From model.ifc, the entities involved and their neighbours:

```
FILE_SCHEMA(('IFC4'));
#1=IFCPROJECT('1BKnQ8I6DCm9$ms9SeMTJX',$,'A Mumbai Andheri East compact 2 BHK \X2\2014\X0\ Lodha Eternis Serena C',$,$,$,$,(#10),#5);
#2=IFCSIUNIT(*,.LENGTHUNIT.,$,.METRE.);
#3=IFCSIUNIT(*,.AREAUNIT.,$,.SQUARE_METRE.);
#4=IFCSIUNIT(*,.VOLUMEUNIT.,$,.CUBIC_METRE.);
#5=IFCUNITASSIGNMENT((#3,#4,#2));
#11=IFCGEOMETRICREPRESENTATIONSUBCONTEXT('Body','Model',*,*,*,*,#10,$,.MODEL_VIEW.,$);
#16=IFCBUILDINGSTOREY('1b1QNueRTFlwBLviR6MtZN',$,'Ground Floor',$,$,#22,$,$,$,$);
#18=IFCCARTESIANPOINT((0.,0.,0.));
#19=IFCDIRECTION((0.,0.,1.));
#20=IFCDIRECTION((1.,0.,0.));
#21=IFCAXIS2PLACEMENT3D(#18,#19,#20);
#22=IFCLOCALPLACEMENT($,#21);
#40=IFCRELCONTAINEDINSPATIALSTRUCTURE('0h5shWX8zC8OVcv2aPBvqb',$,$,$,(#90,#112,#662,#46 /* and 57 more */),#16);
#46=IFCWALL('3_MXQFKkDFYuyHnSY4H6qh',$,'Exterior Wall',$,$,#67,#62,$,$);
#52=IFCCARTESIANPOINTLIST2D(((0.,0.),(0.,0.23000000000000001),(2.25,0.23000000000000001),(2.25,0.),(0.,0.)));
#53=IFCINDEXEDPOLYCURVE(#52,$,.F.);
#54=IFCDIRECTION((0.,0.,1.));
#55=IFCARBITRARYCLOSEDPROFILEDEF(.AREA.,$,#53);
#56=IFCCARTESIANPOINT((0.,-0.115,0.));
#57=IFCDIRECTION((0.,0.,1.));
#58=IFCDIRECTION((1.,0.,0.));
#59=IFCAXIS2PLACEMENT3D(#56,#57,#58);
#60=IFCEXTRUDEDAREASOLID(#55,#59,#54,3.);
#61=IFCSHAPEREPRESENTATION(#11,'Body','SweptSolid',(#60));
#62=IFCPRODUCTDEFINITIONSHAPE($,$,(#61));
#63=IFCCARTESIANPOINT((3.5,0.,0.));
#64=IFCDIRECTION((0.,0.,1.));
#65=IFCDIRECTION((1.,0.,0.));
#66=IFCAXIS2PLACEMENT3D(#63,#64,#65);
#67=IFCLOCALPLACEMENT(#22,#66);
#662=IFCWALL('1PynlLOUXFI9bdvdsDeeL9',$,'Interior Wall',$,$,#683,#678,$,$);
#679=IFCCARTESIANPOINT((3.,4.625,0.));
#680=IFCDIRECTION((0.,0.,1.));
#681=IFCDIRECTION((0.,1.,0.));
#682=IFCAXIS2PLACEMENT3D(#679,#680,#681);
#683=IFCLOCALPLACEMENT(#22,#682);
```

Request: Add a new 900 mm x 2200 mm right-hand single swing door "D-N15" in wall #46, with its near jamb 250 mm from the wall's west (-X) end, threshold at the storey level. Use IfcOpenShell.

```python
import numpy as np
import ifcopenshell
import ifcopenshell.api.feature
import ifcopenshell.api.geometry
import ifcopenshell.api.root
import ifcopenshell.api.spatial
import ifcopenshell.geom
import ifcopenshell.util.element
import ifcopenshell.util.placement
import ifcopenshell.util.representation
import ifcopenshell.util.shape
import ifcopenshell.util.unit

model = ifcopenshell.open("model.ifc")
unit_scale = ifcopenshell.util.unit.calculate_unit_scale(model)
settings = ifcopenshell.geom.settings()


def volume(element):
    """Net volume in cubic metres, openings subtracted."""
    shape = ifcopenshell.geom.create_shape(settings, element)
    return ifcopenshell.util.shape.get_volume(shape.geometry)


wall = model.by_guid("3_MXQFKkDFYuyHnSY4H6qh")
storey = ifcopenshell.util.element.get_container(wall, ifc_class="IfcBuildingStorey")
context = ifcopenshell.util.representation.get_context(model, "Model", "Body", "MODEL_VIEW")
before = volume(wall)

width, height, from_end, sill = 0.9, 2.2, 0.25, 0.0  # metres

# The wall runs along its own X axis, and the end named is its -X end.
wall_shape = ifcopenshell.geom.create_shape(settings, wall)
x, y, z = ifcopenshell.util.shape.get_vertices(wall_shape.geometry).T
start = x.min() + from_end
face, thickness = float(y.min()), float(y.max() - y.min())
wall_matrix = ifcopenshell.util.placement.get_local_placement(wall.ObjectPlacement)
level = ifcopenshell.util.placement.get_local_placement(storey.ObjectPlacement)[2, 3]


def in_wall(x, y):
    """Placement at x, y metres in the wall's axes, at sill height."""
    matrix = wall_matrix.copy()
    matrix[:, 3] = wall_matrix @ np.array([x / unit_scale, y / unit_scale, 0.0, 1.0])
    matrix[2, 3] = level + sill / unit_scale
    return matrix


# Opening: a box that overshoots both wall faces by 50 mm.
opening = ifcopenshell.api.root.create_entity(model, ifc_class="IfcOpeningElement", predefined_type="OPENING")
box = ifcopenshell.api.geometry.add_wall_representation(
    model, context=context, length=width, height=height, thickness=thickness + 0.1
)
ifcopenshell.api.geometry.assign_representation(model, product=opening, representation=box)
ifcopenshell.api.geometry.edit_object_placement(model, product=opening, matrix=in_wall(start, face - 0.05), is_si=False)
ifcopenshell.api.feature.add_feature(model, feature=opening, element=wall)

door = ifcopenshell.api.root.create_entity(model, ifc_class="IfcDoor", name="D-N15", predefined_type="DOOR")
door.OverallWidth, door.OverallHeight = width / unit_scale, height / unit_scale
door.OperationType = "SINGLE_SWING_RIGHT"
body = ifcopenshell.api.geometry.add_door_representation(
    model,
    context=context,
    overall_width=door.OverallWidth,
    overall_height=door.OverallHeight,
    operation_type="SINGLE_SWING_RIGHT",
    lining_properties={"LiningDepth": thickness / unit_scale, "ThresholdDepth": thickness / unit_scale},
)
ifcopenshell.api.geometry.assign_representation(model, product=door, representation=body)
ifcopenshell.api.spatial.assign_container(model, products=[door], relating_structure=storey)
ifcopenshell.api.feature.add_filling(model, opening=opening, element=door)

# The lining spans the wall, so the door starts at the wall face.
ifcopenshell.api.geometry.edit_object_placement(model, product=door, matrix=in_wall(start, face), is_si=False)

after = volume(wall)

print(f"wall volume {before:.3f} -> {after:.3f} m3")

model.write("model_rev.ifc")
```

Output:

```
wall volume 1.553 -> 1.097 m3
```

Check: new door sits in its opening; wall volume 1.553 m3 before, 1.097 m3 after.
